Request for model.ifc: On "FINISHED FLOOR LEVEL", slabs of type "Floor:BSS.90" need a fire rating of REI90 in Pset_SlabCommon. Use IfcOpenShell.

First a look at what the model holds.

```python
import ifcopenshell
import ifcopenshell.util.element

model = ifcopenshell.open("model.ifc")
print(model.schema)
storey = next(s for s in model.by_type("IfcBuildingStorey") if s.Name == "FINISHED FLOOR LEVEL")
slabs = [e for e in ifcopenshell.util.element.get_decomposition(storey) if e.is_a("IfcSlab")]
seen = {}
for e in slabs:
    element_type = ifcopenshell.util.element.get_type(e)
    key = (element_type.Name if element_type != e and element_type else None, ifcopenshell.util.element.get_pset(e, "Pset_SlabCommon", "FireRating"))
    seen[key] = seen.get(key, 0) + 1
for (name, value), count in sorted(seen.items(), key=str):
    print(count, "x", name, "|", value)
```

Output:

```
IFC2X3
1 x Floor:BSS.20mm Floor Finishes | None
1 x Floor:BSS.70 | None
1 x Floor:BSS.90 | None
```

```python
import ifcopenshell
import ifcopenshell.api.pset
import ifcopenshell.util.element

model = ifcopenshell.open("model.ifc")

storey = next(s for s in model.by_type("IfcBuildingStorey") if s.Name == "FINISHED FLOOR LEVEL")
slabs = [e for e in ifcopenshell.util.element.get_decomposition(storey) if e.is_a("IfcSlab")]

count = 0
for e in slabs:
    element_type = ifcopenshell.util.element.get_type(e)
    if element_type in (None, e) or element_type.Name != "Floor:BSS.90":
        continue
    # add_pset returns the element's existing set when there is one.
    pset = ifcopenshell.api.pset.add_pset(model, product=e, name="Pset_SlabCommon")
    ifcopenshell.api.pset.edit_pset(model, pset=pset, properties={"FireRating": "REI90"})
    count += 1

print(count, "slabs updated")

model.write("model_rev.ifc")
```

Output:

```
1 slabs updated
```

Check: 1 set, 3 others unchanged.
